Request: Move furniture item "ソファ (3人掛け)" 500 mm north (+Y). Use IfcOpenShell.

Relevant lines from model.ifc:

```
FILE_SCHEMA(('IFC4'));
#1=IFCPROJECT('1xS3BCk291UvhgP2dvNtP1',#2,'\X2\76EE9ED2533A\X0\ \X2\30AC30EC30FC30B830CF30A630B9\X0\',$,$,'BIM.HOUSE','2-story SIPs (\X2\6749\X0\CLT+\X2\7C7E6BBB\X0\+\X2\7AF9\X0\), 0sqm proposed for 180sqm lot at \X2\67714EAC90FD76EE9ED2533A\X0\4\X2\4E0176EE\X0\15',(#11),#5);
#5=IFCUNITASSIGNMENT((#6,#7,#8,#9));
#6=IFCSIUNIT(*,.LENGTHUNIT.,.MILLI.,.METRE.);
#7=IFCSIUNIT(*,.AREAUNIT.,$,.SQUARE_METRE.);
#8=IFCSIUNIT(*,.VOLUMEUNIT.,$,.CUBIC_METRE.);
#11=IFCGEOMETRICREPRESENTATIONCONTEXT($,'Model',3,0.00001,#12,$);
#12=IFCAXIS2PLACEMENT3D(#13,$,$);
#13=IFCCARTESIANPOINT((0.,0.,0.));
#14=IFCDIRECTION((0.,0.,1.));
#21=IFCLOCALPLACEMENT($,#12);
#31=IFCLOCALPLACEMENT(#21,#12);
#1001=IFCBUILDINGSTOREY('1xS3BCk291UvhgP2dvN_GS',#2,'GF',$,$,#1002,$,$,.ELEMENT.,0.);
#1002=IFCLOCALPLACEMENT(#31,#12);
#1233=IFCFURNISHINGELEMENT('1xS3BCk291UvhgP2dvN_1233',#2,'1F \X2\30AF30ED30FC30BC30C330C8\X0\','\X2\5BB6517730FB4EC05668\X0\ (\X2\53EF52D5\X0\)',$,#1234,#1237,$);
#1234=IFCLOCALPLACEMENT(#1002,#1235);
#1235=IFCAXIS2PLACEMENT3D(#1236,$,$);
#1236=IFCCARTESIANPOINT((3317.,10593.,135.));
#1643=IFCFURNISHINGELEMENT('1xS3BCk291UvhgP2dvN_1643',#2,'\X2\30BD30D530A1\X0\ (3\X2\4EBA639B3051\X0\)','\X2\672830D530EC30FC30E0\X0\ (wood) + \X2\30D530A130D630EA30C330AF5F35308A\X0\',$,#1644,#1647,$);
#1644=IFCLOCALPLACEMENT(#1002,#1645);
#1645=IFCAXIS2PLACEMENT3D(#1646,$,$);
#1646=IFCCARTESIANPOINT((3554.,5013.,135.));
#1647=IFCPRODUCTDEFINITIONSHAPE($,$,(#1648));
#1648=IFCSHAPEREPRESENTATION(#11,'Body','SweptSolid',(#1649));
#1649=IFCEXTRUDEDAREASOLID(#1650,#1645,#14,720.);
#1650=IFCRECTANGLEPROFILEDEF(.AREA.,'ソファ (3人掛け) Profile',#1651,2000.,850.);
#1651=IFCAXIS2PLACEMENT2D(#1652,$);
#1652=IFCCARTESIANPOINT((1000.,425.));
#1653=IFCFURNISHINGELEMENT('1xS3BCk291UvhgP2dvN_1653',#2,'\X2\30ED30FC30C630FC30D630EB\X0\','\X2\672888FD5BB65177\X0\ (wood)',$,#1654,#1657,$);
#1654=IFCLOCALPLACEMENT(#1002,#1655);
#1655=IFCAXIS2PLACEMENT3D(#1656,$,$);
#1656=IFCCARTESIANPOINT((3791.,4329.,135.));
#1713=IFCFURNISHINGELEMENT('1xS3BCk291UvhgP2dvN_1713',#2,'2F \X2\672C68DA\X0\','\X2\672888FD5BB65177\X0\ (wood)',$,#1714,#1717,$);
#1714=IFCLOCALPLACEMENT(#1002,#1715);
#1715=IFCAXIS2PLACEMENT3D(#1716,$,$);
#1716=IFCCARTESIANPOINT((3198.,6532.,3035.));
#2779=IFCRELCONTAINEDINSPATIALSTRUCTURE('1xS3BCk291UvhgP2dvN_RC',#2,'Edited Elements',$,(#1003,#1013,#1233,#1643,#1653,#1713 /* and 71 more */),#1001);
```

```python
import ifcopenshell
import ifcopenshell.api.geometry
import ifcopenshell.util.placement

model = ifcopenshell.open("model.ifc")

item = model.by_guid("1xS3BCk291UvhgP2dvN_1643")
matrix = ifcopenshell.util.placement.get_local_placement(item.ObjectPlacement)
matrix[1, 3] += 500.0
ifcopenshell.api.geometry.edit_object_placement(model, product=item, matrix=matrix, is_si=False)

print(ifcopenshell.util.placement.get_local_placement(item.ObjectPlacement).round(3) + 0.0)

model.write("model_updated.ifc")
```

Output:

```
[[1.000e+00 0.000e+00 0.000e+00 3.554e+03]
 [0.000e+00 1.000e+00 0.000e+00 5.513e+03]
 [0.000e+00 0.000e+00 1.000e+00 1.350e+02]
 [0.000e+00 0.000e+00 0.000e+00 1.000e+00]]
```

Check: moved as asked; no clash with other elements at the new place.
